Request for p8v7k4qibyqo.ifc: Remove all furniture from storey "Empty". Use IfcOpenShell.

First a look at what the model holds.

```python
import ifcopenshell
import ifcopenshell.util.element

model = ifcopenshell.open("p8v7k4qibyqo.ifc")
print(model.schema)
storey = next(s for s in model.by_type("IfcBuildingStorey") if s.Name == "Empty")
furniture = [e for e in ifcopenshell.util.element.get_decomposition(storey) if e.is_a("IfcFurnishingElement")]
seen = {}
for e in furniture:
    element_type = ifcopenshell.util.element.get_type(e)
    name = element_type.Name if element_type not in (None, e) else None
    seen[name] = seen.get(name, 0) + 1
for name, count in sorted(seen.items(), key=str):
    print(count, "x", name)
```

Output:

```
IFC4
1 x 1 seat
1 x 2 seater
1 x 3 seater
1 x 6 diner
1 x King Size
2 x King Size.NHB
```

```python
import ifcopenshell
import ifcopenshell.api.root
import ifcopenshell.util.element

model = ifcopenshell.open("p8v7k4qibyqo.ifc")

storey = next(s for s in model.by_type("IfcBuildingStorey") if s.Name == "Empty")
furniture = [e for e in ifcopenshell.util.element.get_decomposition(storey) if e.is_a("IfcFurnishingElement")]

for e in furniture:
    ifcopenshell.api.root.remove_product(model, product=e)
print(len(furniture), "removed")

model.write("p8v7k4qibyqo_edited.ifc")
```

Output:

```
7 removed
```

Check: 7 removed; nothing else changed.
